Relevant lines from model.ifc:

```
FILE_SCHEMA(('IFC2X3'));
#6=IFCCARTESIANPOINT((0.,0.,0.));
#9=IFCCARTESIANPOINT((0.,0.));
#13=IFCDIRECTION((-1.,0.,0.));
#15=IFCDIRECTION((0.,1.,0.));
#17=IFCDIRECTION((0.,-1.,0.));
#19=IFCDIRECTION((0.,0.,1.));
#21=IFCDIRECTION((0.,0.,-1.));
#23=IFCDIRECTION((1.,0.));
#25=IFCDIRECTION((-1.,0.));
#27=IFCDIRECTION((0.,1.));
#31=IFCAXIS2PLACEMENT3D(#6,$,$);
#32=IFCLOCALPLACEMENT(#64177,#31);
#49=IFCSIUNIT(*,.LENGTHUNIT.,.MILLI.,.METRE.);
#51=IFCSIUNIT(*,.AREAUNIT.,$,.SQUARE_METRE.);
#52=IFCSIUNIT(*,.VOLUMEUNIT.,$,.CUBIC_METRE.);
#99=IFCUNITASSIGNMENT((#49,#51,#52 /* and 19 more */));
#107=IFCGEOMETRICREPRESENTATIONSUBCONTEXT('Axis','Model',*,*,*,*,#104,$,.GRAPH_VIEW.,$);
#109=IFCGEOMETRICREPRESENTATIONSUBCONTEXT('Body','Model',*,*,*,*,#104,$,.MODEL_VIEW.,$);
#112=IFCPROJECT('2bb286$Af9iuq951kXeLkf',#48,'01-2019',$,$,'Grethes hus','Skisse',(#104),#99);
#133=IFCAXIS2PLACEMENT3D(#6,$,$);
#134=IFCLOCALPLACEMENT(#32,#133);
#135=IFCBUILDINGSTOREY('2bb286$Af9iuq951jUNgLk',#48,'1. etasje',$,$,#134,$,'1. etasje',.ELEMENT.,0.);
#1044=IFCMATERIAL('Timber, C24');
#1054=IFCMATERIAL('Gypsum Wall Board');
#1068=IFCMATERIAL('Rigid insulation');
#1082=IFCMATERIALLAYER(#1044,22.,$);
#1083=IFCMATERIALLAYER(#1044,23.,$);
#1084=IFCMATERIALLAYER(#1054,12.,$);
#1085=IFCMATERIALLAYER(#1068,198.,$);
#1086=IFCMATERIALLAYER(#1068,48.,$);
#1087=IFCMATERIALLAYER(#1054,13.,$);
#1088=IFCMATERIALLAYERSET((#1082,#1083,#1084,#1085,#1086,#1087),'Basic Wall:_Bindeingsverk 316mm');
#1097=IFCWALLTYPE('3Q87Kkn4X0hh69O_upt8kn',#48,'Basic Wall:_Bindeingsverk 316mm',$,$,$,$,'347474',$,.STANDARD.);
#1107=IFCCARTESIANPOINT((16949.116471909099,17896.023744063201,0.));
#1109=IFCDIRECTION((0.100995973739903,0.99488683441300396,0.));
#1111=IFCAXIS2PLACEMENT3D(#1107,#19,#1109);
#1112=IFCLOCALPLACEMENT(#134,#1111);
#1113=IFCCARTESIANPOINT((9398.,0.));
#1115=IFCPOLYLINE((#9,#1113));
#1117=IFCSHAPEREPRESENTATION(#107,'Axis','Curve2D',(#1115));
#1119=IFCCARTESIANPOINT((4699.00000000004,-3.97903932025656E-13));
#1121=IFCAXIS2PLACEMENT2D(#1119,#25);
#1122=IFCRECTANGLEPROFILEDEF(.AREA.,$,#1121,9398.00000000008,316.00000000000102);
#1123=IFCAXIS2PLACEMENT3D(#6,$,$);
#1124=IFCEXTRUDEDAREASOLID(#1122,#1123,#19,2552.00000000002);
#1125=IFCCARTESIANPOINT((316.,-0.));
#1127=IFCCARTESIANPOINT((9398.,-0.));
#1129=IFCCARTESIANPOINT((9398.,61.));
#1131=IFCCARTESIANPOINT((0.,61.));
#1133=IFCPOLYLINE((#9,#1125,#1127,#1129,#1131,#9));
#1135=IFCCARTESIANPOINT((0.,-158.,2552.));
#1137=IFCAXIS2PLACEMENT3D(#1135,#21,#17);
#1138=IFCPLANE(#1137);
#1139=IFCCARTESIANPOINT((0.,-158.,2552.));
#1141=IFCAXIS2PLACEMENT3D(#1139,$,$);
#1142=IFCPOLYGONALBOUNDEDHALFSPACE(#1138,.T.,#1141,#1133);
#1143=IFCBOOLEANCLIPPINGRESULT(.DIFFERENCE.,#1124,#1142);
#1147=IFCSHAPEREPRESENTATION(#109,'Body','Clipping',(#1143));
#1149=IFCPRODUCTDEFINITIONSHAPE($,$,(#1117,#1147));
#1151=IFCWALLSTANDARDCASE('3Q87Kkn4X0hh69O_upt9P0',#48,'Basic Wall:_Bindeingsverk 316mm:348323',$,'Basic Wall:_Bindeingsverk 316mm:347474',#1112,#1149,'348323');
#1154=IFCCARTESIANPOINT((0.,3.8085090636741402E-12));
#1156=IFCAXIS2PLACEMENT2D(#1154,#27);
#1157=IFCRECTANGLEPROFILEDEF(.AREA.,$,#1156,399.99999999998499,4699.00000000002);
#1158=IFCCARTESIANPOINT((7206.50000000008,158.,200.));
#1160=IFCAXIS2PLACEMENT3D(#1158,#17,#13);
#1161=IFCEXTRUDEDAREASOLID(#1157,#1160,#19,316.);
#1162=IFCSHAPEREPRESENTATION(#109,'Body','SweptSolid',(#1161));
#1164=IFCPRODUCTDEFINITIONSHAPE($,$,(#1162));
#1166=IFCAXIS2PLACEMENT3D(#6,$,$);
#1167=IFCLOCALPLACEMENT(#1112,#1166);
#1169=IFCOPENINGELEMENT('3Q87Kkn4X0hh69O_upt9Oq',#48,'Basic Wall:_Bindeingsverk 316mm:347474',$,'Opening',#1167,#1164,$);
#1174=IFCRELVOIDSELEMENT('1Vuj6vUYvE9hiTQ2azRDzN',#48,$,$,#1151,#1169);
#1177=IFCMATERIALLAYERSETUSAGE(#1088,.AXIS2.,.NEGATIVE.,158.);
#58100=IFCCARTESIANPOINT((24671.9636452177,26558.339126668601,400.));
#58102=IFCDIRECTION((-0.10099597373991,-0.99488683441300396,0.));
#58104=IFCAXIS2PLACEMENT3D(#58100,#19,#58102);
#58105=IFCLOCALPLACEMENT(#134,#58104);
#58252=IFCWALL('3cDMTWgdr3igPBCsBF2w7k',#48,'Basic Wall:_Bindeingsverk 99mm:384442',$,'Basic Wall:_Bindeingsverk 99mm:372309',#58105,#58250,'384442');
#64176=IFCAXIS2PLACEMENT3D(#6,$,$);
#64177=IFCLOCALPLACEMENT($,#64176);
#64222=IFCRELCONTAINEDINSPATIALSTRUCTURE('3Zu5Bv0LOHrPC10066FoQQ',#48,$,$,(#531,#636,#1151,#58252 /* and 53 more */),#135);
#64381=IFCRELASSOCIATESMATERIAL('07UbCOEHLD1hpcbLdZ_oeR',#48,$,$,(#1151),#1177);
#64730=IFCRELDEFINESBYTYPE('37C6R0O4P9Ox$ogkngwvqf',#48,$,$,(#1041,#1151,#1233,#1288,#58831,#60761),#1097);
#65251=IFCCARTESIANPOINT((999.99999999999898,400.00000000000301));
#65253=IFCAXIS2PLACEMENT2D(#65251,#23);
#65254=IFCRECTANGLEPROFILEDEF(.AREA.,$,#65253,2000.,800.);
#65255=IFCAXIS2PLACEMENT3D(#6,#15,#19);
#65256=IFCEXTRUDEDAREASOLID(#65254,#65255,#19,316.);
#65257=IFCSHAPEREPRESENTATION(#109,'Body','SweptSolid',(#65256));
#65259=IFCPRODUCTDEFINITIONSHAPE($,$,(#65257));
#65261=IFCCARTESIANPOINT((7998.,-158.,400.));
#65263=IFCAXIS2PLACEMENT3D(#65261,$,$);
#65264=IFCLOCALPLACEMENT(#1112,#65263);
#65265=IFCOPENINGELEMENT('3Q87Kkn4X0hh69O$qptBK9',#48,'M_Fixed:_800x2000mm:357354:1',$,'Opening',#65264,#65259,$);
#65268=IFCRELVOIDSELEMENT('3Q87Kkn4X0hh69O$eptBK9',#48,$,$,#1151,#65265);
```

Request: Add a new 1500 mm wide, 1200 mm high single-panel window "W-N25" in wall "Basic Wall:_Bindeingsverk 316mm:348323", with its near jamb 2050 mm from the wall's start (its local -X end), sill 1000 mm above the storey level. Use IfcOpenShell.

```python
import numpy as np
import ifcopenshell
import ifcopenshell.api.feature
import ifcopenshell.api.geometry
import ifcopenshell.api.root
import ifcopenshell.api.spatial
import ifcopenshell.api.type
import ifcopenshell.geom
import ifcopenshell.util.element
import ifcopenshell.util.placement
import ifcopenshell.util.representation
import ifcopenshell.util.shape
import ifcopenshell.util.unit

model = ifcopenshell.open("model.ifc")
unit_scale = ifcopenshell.util.unit.calculate_unit_scale(model)
settings = ifcopenshell.geom.settings()


def volume(element):
    """Net volume in cubic metres, openings subtracted."""
    shape = ifcopenshell.geom.create_shape(settings, element)
    return ifcopenshell.util.shape.get_volume(shape.geometry)


wall = model.by_id(1151)
storey = ifcopenshell.util.element.get_container(wall, ifc_class="IfcBuildingStorey")
context = ifcopenshell.util.representation.get_context(model, "Model", "Body", "MODEL_VIEW")
before = volume(wall)

width, height, from_end, sill = 1.5, 1.2, 2.05, 1  # metres

# The wall runs along its own X axis, and the end named is its -X end.
wall_shape = ifcopenshell.geom.create_shape(settings, wall)
x, y, z = ifcopenshell.util.shape.get_vertices(wall_shape.geometry).T
start = x.min() + from_end
face, thickness = float(y.min()), float(y.max() - y.min())
wall_matrix = ifcopenshell.util.placement.get_local_placement(wall.ObjectPlacement)
level = ifcopenshell.util.placement.get_local_placement(storey.ObjectPlacement)[2, 3]


def in_wall(x, y):
    """Placement at x, y metres in the wall's axes, at sill height."""
    matrix = wall_matrix.copy()
    matrix[:, 3] = wall_matrix @ np.array([x / unit_scale, y / unit_scale, 0.0, 1.0])
    matrix[2, 3] = level + sill / unit_scale
    return matrix


# Opening: a box that overshoots both wall faces by 50 mm.
opening = ifcopenshell.api.root.create_entity(model, ifc_class="IfcOpeningElement")
box = ifcopenshell.api.geometry.add_wall_representation(
    model, context=context, length=width, height=height, thickness=thickness + 0.1
)
ifcopenshell.api.geometry.assign_representation(model, product=opening, representation=box)
ifcopenshell.api.geometry.edit_object_placement(model, product=opening, matrix=in_wall(start, face - 0.05), is_si=False)
ifcopenshell.api.feature.add_feature(model, feature=opening, element=wall)

window = ifcopenshell.api.root.create_entity(model, ifc_class="IfcWindow", name="W-N25")
window.OverallWidth, window.OverallHeight = width / unit_scale, height / unit_scale
body = ifcopenshell.api.geometry.add_window_representation(
    model,
    context=context,
    overall_width=window.OverallWidth,
    overall_height=window.OverallHeight,
    partition_type="SINGLE_PANEL",
)
ifcopenshell.api.geometry.assign_representation(model, product=window, representation=body)
ifcopenshell.api.spatial.assign_container(model, products=[window], relating_structure=storey)
fills = ifcopenshell.api.feature.add_filling(model, opening=opening, element=window)
fills.OwnerHistory = window.OwnerHistory  # required in IFC2X3

# IFC2X3 keeps the operation on the window style.
style = ifcopenshell.api.root.create_entity(model, ifc_class="IfcWindowStyle", name="W-N25")
style.OperationType, style.ConstructionType = "SINGLE_PANEL", "NOTDEFINED"
style.ParameterTakesPrecedence = style.Sizeable = False
ifcopenshell.api.type.assign_type(model, related_objects=[window], relating_type=style)

# Centre the window in the wall's thickness.
ifcopenshell.api.geometry.edit_object_placement(model, product=window, matrix=in_wall(start, face), is_si=False)
window_shape = ifcopenshell.geom.create_shape(settings, window)
depth = ifcopenshell.util.shape.get_vertices(window_shape.geometry)[:, 1]
offset = face + thickness / 2 - (depth.min() + depth.max()) / 2
ifcopenshell.api.geometry.edit_object_placement(model, product=window, matrix=in_wall(start, offset), is_si=False)

after = volume(wall)

print(f"wall volume {before:.3f} -> {after:.3f} m3")

model.write("model_rev.ifc")
```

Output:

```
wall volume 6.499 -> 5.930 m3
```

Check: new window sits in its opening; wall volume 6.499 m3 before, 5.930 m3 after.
